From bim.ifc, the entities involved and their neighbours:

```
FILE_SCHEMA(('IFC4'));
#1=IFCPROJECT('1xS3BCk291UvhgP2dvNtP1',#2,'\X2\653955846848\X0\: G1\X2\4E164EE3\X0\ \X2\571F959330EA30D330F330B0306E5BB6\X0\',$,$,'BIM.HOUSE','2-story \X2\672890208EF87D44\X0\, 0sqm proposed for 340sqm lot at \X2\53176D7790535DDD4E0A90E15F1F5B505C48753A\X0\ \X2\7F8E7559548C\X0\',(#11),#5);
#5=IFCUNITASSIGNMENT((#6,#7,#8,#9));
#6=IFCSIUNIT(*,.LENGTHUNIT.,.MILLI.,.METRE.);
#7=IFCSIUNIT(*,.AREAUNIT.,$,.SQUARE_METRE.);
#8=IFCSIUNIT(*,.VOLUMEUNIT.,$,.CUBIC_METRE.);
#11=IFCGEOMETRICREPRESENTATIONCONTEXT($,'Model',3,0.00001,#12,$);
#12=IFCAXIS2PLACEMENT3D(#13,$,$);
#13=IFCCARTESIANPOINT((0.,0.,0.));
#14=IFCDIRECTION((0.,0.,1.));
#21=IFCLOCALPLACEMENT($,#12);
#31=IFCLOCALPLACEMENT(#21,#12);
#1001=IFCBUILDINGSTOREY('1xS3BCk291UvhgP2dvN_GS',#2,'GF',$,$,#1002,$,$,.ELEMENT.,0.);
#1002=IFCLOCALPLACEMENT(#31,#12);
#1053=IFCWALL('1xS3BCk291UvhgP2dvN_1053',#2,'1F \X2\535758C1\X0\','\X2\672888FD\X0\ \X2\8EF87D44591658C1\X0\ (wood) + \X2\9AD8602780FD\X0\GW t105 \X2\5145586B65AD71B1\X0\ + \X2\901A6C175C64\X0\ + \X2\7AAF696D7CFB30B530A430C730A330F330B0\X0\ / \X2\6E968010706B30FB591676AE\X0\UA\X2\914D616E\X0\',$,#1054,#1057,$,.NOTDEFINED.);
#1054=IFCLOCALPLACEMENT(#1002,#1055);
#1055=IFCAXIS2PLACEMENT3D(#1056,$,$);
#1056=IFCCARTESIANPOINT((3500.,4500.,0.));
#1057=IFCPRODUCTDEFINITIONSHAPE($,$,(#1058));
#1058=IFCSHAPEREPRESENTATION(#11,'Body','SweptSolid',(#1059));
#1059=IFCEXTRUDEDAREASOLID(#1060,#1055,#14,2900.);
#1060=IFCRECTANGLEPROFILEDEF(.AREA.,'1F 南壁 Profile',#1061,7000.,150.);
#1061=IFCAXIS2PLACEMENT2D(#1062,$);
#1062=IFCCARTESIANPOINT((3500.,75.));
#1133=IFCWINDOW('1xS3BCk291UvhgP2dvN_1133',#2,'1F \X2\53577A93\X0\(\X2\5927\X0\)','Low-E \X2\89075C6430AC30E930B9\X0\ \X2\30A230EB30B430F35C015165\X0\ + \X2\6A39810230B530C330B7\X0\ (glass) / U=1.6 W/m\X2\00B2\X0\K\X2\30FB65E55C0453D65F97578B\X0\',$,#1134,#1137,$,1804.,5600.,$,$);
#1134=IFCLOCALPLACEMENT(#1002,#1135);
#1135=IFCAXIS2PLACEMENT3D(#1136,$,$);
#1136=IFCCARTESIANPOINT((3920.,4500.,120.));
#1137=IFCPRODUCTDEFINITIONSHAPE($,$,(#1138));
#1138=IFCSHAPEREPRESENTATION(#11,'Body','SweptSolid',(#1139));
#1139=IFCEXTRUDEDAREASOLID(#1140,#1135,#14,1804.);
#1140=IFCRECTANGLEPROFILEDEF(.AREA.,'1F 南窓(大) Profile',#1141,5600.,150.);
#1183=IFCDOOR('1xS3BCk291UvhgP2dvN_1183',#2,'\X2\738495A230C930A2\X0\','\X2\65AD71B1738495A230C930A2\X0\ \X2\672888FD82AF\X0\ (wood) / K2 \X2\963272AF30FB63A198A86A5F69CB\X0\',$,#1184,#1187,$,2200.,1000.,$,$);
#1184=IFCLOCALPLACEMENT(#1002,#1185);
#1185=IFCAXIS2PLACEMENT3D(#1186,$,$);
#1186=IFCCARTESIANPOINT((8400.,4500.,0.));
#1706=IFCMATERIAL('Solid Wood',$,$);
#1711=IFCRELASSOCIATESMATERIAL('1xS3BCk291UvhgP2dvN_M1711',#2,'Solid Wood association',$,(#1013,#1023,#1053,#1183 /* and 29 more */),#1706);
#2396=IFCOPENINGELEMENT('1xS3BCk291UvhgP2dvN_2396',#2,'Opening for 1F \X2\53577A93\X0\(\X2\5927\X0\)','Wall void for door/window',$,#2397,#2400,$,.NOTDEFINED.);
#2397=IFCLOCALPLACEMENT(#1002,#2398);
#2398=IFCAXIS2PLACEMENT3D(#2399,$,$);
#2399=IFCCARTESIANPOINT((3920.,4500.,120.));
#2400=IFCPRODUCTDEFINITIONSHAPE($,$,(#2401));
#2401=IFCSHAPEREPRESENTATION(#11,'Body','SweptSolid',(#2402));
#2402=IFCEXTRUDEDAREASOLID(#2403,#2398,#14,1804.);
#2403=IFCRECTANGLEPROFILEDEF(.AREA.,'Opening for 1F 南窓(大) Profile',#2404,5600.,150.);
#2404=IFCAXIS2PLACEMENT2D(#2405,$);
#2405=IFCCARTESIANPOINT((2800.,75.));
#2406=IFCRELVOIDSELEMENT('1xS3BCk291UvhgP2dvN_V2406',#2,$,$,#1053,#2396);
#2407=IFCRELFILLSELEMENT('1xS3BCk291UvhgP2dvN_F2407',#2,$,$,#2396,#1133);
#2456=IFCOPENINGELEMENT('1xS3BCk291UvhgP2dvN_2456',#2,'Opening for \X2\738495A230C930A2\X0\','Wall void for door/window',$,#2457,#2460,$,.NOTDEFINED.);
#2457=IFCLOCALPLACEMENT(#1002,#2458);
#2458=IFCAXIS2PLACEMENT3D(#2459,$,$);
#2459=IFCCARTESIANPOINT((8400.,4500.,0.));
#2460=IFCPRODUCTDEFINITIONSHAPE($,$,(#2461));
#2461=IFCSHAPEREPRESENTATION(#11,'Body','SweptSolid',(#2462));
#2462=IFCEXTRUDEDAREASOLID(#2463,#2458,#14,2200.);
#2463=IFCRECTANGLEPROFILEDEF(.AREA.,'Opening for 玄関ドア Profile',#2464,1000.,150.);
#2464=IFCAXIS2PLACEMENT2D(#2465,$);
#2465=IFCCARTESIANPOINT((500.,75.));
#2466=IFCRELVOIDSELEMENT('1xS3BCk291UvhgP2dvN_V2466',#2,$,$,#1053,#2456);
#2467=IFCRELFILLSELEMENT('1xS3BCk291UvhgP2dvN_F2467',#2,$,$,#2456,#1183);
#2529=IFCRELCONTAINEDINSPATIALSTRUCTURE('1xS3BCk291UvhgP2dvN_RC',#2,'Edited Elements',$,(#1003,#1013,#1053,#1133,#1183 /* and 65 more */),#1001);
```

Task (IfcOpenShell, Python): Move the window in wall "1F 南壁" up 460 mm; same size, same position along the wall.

```python
import numpy as np
import ifcopenshell
import ifcopenshell.api.geometry
import ifcopenshell.util.placement
import ifcopenshell.util.unit

model = ifcopenshell.open("bim.ifc")
unit_scale = ifcopenshell.util.unit.calculate_unit_scale(model)

window = model.by_guid("1xS3BCk291UvhgP2dvN_1133")
opening = window.FillsVoids[0].RelatingOpeningElement
dz = 460.0

shift = np.array([0.0, 0.0, dz])
# The window is not placed relative to its opening, so move both.
for product in (opening, window):
    matrix = ifcopenshell.util.placement.get_local_placement(product.ObjectPlacement)
    matrix[:3, 3] += shift
    ifcopenshell.api.geometry.edit_object_placement(model, product=product, matrix=matrix, is_si=False)

print(f"moved by {dz * unit_scale:+.3f} m")

model.write("bim_rev.ifc")
```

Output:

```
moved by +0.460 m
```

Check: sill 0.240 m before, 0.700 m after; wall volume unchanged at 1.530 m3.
